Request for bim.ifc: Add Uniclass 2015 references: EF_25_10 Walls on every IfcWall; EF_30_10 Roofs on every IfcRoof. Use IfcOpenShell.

First a look at what the model holds.

```python
import ifcopenshell

model = ifcopenshell.open("bim.ifc")
print(model.schema)
print("classifications:", [c.Name for c in model.by_type("IfcClassification")])
for ifc_class in ("IfcDoor", "IfcRoof", "IfcStair", "IfcWall", "IfcWindow"):
    print(ifc_class, len(model.by_type(ifc_class)))
```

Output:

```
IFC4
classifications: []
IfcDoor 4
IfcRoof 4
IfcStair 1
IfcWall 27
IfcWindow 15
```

```python
import ifcopenshell
import ifcopenshell.api.classification

model = ifcopenshell.open("bim.ifc")

system = ifcopenshell.api.classification.add_classification(model, classification="Uniclass 2015")

codes = {
    "IfcWall": ("EF_25_10", "Walls"),
    "IfcRoof": ("EF_30_10", "Roofs"),
}
for ifc_class, (code, name) in codes.items():
    products = model.by_type(ifc_class)
    ifcopenshell.api.classification.add_reference(
        model, products=products, classification=system, identification=code, name=name
    )
    print(code, len(products))

model.write("bim_updated.ifc")
```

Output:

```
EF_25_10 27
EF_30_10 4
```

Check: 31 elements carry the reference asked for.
